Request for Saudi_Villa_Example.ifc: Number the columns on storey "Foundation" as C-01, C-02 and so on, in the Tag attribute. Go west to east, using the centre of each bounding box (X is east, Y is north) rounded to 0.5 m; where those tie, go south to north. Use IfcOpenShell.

First a look at what the model holds.

```python
import ifcopenshell
import ifcopenshell.util.element
import ifcopenshell.util.placement

model = ifcopenshell.open("Saudi_Villa_Example.ifc")
print(model.schema)
storey = next(s for s in model.by_type("IfcBuildingStorey") if s.Name == "Foundation")
columns = [e for e in ifcopenshell.util.element.get_decomposition(storey) if e.is_a("IfcColumn")]
for e in sorted(columns, key=lambda e: e.id()):
    origin = ifcopenshell.util.placement.get_local_placement(e.ObjectPlacement)[:3, 3]
    print(e.id(), e.Tag, e.Name, origin.round(2) + 0.0, sep=" | ")
```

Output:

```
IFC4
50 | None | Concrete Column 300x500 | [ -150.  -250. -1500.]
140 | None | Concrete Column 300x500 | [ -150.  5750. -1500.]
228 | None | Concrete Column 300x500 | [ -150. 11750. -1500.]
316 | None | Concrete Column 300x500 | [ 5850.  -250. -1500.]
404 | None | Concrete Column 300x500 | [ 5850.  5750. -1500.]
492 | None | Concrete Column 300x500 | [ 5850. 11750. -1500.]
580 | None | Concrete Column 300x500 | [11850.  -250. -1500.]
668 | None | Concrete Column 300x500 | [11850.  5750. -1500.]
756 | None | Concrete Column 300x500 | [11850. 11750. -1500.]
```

```python
import ifcopenshell
import ifcopenshell.geom
import ifcopenshell.util.element
import ifcopenshell.util.shape

model = ifcopenshell.open("Saudi_Villa_Example.ifc")
settings = ifcopenshell.geom.settings()
settings.set("use-world-coords", True)


def centre(element):
    shape = ifcopenshell.geom.create_shape(settings, element)
    return ifcopenshell.util.shape.get_bbox_centroid(shape.geometry)


storey = next(s for s in model.by_type("IfcBuildingStorey") if s.Name == "Foundation")
columns = [e for e in ifcopenshell.util.element.get_decomposition(storey) if e.is_a("IfcColumn")]

# Insertion points can sit at a corner or the storey origin, so sort by the geometry (in metres).
centres = {e: centre(e) for e in columns}
columns.sort(key=lambda e: (round(centres[e][0] / 0.5), centres[e][1]))

for i, e in enumerate(columns, start=1):
    number = f"C-{i:02d}"
    e.Tag = number
    print(e.id(), number)

model.write("Saudi_Villa_Example-out.ifc")
```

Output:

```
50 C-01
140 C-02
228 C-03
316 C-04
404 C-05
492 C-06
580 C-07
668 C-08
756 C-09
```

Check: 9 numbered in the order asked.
